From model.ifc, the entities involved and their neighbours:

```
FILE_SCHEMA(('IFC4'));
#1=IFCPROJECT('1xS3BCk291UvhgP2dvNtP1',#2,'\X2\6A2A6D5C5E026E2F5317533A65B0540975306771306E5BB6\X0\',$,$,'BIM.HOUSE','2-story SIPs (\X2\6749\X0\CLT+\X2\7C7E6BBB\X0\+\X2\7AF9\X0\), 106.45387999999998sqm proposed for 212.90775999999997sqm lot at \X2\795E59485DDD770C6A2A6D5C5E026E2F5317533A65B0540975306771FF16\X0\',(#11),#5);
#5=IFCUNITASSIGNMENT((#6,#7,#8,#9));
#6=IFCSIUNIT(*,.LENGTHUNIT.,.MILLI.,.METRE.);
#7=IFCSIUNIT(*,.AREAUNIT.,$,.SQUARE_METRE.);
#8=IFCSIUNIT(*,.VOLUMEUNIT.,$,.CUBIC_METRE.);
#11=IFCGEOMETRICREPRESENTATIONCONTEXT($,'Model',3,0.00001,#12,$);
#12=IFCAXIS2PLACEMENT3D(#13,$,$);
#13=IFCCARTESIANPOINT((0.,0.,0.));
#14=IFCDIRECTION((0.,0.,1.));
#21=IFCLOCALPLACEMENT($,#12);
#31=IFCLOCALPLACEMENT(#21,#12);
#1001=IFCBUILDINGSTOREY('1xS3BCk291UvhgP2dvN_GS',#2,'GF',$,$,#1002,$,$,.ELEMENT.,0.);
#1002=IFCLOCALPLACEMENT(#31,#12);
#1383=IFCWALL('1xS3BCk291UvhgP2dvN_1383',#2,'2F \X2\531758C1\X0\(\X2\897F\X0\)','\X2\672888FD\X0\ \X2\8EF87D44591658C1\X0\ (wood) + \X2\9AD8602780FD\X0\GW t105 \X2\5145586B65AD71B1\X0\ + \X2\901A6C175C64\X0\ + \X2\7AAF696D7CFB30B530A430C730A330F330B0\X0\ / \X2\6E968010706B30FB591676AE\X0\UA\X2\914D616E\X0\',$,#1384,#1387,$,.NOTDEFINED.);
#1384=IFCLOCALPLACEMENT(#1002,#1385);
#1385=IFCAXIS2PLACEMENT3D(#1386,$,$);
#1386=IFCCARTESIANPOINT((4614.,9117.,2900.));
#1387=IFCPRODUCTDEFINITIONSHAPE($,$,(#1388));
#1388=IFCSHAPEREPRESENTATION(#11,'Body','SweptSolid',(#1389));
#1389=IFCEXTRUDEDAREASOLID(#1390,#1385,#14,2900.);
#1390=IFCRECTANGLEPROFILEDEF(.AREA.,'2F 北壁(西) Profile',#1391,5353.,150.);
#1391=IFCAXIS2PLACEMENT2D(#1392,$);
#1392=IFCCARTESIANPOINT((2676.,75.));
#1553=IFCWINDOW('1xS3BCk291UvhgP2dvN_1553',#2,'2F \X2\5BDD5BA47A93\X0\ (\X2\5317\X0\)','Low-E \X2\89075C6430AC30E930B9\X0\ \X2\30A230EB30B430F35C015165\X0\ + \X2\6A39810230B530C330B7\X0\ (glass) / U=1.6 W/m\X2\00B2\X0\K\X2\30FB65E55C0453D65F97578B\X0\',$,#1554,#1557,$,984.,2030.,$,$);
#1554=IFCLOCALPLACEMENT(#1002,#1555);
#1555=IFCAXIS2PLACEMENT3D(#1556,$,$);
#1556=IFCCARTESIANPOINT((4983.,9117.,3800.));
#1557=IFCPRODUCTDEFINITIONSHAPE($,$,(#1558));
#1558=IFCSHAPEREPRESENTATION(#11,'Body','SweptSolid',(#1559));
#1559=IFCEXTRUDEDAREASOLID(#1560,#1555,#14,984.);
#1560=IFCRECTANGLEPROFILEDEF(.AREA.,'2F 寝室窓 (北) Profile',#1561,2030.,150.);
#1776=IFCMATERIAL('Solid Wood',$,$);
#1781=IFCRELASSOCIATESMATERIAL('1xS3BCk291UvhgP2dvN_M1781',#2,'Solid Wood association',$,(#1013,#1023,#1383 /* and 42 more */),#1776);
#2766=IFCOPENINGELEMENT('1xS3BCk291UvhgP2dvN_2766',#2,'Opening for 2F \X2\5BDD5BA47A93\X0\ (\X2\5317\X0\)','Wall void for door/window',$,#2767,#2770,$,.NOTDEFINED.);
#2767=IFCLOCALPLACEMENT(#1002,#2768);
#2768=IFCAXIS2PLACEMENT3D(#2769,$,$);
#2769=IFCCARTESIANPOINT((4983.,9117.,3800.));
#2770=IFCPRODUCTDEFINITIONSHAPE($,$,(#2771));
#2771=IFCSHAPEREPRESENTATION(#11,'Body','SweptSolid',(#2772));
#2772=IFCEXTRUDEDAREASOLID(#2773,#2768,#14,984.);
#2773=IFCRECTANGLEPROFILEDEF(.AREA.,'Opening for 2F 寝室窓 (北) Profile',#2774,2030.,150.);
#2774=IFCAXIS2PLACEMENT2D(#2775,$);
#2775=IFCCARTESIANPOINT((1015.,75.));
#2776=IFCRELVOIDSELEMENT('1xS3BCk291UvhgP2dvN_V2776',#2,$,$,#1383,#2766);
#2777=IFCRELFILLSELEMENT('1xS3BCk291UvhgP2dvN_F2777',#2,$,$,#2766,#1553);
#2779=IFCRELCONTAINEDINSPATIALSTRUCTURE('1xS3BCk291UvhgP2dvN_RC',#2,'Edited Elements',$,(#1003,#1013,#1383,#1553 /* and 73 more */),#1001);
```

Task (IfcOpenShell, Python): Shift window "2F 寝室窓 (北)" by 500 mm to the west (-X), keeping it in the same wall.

```python
import ifcopenshell
import ifcopenshell.api.geometry
import ifcopenshell.util.placement

model = ifcopenshell.open("model.ifc")

window = model.by_guid("1xS3BCk291UvhgP2dvN_1553")
opening = window.FillsVoids[0].RelatingOpeningElement
wall = opening.VoidsElements[0].RelatingBuildingElement

wall_matrix = ifcopenshell.util.placement.get_local_placement(wall.ObjectPlacement)
shift = wall_matrix[:3, 0] * -500.0
before = ifcopenshell.util.placement.get_local_placement(window.ObjectPlacement)[:3, 3].copy()

# The window is not placed relative to its opening, so move both.
for product in (opening, window):
    matrix = ifcopenshell.util.placement.get_local_placement(product.ObjectPlacement)
    matrix[:3, 3] += shift
    ifcopenshell.api.geometry.edit_object_placement(model, product=product, matrix=matrix, is_si=False)

after = ifcopenshell.util.placement.get_local_placement(window.ObjectPlacement)[:3, 3]
print("window moved by", (after - before).round(3) + 0.0)

model.write("model-out.ifc")
```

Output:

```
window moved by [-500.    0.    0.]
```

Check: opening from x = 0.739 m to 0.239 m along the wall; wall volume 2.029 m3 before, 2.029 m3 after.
